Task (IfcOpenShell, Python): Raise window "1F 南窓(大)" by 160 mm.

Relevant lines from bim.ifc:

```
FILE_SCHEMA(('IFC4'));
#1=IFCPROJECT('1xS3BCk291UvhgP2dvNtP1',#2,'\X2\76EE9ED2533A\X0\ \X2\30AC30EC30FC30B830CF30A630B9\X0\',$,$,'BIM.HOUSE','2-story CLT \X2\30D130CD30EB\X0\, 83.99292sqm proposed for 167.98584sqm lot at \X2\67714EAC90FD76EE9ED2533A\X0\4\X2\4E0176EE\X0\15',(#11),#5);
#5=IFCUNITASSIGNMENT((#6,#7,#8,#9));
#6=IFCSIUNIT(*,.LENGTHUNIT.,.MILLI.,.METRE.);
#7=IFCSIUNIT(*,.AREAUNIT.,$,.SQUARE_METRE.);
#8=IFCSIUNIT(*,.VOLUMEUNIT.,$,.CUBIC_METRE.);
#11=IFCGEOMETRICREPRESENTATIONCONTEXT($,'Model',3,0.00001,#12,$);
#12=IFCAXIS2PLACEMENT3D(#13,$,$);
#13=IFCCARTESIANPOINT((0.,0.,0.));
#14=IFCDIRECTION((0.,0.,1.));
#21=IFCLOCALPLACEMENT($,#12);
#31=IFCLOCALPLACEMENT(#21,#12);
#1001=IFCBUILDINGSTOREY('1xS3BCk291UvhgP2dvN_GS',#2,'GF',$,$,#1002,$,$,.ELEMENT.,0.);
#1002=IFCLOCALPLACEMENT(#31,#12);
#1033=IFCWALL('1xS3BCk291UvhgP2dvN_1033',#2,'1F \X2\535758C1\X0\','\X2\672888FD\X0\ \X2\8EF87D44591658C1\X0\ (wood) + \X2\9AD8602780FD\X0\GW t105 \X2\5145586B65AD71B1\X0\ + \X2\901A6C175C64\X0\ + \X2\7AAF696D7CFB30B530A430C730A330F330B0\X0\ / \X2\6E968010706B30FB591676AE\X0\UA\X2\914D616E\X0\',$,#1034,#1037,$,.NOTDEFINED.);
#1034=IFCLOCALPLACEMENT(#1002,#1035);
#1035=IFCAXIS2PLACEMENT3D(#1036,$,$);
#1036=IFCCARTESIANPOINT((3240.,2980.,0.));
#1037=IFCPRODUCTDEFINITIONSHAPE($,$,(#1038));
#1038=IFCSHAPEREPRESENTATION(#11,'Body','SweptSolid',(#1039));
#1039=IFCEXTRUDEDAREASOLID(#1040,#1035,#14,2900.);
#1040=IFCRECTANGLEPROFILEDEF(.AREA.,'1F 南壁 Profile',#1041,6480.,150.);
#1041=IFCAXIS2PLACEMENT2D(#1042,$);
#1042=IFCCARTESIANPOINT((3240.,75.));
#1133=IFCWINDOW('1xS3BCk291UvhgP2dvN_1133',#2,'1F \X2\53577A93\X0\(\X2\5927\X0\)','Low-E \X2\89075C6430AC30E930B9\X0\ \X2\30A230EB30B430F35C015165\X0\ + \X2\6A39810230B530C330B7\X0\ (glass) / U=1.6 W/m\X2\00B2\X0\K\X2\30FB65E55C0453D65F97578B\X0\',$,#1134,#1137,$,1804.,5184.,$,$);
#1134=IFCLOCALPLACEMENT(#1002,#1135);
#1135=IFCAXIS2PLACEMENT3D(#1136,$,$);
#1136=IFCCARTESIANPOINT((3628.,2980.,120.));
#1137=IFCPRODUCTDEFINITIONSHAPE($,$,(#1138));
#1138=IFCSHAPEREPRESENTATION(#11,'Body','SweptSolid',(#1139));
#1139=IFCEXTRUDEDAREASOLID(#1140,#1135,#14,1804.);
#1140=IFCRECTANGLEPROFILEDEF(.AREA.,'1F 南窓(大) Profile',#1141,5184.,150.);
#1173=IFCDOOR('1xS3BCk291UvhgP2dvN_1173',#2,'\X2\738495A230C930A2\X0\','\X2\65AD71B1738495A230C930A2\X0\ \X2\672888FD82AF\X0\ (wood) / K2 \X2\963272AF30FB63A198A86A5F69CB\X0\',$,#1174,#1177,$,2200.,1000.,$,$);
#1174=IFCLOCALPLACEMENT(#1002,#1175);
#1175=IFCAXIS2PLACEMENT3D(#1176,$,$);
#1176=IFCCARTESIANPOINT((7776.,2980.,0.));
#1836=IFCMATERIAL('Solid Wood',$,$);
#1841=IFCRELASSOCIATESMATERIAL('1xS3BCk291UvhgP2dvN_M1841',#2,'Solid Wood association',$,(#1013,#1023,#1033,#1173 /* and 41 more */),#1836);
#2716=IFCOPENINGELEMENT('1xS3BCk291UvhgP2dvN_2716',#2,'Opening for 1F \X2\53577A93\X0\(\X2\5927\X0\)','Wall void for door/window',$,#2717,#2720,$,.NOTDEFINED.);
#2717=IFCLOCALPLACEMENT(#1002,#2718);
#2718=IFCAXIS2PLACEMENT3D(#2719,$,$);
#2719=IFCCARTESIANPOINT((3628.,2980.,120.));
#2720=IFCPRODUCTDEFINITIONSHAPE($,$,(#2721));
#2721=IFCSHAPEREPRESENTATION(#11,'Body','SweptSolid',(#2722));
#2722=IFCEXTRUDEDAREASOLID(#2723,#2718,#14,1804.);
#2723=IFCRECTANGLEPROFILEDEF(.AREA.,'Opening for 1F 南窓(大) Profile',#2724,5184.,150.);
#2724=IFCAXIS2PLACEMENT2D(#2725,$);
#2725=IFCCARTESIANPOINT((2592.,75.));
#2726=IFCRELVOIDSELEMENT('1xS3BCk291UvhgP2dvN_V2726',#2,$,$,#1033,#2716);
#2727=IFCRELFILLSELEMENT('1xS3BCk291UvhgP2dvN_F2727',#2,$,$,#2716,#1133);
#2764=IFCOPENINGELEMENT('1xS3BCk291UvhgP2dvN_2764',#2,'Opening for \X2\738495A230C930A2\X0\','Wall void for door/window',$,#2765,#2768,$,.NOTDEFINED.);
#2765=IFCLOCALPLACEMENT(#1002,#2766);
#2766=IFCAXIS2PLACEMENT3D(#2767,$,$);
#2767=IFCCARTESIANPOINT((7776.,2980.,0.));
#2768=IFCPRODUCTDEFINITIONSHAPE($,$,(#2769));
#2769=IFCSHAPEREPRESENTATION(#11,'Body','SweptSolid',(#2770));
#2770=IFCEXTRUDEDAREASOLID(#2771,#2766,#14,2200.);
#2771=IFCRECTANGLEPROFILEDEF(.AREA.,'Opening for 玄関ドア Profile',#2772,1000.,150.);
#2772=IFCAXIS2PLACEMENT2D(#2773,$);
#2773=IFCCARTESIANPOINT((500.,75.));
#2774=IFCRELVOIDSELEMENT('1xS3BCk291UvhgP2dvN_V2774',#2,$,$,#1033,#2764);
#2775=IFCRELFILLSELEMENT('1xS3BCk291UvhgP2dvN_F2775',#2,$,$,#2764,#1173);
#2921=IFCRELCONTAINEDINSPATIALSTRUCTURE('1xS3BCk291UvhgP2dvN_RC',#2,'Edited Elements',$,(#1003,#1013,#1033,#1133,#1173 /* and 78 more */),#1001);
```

```python
import numpy as np
import ifcopenshell
import ifcopenshell.api.geometry
import ifcopenshell.util.placement
import ifcopenshell.util.unit

model = ifcopenshell.open("bim.ifc")
unit_scale = ifcopenshell.util.unit.calculate_unit_scale(model)

window = model.by_guid("1xS3BCk291UvhgP2dvN_1133")
opening = window.FillsVoids[0].RelatingOpeningElement
dz = 160.0

shift = np.array([0.0, 0.0, dz])
# The window is not placed relative to its opening, so move both.
for product in (opening, window):
    matrix = ifcopenshell.util.placement.get_local_placement(product.ObjectPlacement)
    matrix[:3, 3] += shift
    ifcopenshell.api.geometry.edit_object_placement(model, product=product, matrix=matrix, is_si=False)

print(f"moved by {dz * unit_scale:+.3f} m")

model.write("bim-out.ifc")
```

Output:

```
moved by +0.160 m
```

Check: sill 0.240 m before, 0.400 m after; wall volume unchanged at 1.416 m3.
